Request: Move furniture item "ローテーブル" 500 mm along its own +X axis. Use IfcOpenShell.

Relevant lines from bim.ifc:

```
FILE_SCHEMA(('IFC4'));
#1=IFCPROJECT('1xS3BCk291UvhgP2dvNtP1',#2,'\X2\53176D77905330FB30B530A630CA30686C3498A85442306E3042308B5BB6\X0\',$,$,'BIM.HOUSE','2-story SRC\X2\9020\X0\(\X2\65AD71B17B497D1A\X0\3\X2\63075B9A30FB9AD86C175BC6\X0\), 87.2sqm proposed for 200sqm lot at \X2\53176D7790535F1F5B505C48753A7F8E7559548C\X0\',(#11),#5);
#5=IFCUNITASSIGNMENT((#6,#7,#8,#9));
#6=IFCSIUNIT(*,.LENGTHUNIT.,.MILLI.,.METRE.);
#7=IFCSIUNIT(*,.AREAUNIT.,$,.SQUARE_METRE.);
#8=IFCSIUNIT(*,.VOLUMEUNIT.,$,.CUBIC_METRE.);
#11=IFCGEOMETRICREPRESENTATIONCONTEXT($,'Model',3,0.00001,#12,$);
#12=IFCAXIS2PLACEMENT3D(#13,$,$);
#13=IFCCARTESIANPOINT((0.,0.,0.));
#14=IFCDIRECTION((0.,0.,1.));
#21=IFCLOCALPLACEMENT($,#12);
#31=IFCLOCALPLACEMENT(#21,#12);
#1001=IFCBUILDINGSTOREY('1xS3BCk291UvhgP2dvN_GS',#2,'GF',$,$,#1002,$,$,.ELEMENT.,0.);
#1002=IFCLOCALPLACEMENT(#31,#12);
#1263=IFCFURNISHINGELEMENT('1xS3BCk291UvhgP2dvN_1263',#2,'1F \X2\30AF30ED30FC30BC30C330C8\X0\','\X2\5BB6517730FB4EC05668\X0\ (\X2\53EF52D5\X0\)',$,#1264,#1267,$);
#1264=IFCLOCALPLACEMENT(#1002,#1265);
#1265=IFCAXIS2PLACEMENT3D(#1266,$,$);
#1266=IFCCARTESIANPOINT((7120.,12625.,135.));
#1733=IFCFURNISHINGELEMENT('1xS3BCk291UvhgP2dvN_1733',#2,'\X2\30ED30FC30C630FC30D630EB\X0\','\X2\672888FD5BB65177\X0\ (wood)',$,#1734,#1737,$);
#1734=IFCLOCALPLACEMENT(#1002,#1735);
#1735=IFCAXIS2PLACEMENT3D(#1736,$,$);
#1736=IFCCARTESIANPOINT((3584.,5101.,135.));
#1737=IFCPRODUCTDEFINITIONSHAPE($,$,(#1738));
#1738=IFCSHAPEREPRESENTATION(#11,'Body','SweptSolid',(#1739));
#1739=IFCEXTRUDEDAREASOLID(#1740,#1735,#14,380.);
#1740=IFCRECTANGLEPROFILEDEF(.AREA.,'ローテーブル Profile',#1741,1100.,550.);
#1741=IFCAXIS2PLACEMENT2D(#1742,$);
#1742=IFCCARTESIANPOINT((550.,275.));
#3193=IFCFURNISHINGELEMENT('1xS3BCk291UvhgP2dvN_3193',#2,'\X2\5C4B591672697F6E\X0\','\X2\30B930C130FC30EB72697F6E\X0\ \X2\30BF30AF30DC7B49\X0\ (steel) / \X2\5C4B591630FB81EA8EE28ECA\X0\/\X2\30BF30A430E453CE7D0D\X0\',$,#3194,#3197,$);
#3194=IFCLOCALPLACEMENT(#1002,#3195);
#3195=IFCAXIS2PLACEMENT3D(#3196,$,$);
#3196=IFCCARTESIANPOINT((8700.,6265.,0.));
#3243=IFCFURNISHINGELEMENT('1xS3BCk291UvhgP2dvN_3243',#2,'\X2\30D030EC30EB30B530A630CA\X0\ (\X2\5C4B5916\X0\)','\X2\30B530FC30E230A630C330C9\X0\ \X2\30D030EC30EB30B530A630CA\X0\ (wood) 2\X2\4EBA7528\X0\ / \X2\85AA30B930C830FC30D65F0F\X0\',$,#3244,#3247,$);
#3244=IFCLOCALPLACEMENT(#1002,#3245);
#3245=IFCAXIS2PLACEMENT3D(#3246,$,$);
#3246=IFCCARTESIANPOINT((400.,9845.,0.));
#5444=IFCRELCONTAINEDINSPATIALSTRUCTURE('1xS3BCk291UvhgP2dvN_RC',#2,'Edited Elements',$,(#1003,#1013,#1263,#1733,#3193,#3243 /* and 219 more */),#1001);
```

```python
import ifcopenshell
import ifcopenshell.api.geometry
import ifcopenshell.util.placement
import ifcopenshell.util.unit

model = ifcopenshell.open("bim.ifc")
unit_scale = ifcopenshell.util.unit.calculate_unit_scale(model)

item = model.by_guid("1xS3BCk291UvhgP2dvN_1733")
matrix = ifcopenshell.util.placement.get_local_placement(item.ObjectPlacement)
matrix[:3, 3] += matrix[:3, 0] * 0.5 / unit_scale
ifcopenshell.api.geometry.edit_object_placement(model, product=item, matrix=matrix, is_si=False)

print(ifcopenshell.util.placement.get_local_placement(item.ObjectPlacement).round(3) + 0.0)

model.write("bim-out.ifc")
```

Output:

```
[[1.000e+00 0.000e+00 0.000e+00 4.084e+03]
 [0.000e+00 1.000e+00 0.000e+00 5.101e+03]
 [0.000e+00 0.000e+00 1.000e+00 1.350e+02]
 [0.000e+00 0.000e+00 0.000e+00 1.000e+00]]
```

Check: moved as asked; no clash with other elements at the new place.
